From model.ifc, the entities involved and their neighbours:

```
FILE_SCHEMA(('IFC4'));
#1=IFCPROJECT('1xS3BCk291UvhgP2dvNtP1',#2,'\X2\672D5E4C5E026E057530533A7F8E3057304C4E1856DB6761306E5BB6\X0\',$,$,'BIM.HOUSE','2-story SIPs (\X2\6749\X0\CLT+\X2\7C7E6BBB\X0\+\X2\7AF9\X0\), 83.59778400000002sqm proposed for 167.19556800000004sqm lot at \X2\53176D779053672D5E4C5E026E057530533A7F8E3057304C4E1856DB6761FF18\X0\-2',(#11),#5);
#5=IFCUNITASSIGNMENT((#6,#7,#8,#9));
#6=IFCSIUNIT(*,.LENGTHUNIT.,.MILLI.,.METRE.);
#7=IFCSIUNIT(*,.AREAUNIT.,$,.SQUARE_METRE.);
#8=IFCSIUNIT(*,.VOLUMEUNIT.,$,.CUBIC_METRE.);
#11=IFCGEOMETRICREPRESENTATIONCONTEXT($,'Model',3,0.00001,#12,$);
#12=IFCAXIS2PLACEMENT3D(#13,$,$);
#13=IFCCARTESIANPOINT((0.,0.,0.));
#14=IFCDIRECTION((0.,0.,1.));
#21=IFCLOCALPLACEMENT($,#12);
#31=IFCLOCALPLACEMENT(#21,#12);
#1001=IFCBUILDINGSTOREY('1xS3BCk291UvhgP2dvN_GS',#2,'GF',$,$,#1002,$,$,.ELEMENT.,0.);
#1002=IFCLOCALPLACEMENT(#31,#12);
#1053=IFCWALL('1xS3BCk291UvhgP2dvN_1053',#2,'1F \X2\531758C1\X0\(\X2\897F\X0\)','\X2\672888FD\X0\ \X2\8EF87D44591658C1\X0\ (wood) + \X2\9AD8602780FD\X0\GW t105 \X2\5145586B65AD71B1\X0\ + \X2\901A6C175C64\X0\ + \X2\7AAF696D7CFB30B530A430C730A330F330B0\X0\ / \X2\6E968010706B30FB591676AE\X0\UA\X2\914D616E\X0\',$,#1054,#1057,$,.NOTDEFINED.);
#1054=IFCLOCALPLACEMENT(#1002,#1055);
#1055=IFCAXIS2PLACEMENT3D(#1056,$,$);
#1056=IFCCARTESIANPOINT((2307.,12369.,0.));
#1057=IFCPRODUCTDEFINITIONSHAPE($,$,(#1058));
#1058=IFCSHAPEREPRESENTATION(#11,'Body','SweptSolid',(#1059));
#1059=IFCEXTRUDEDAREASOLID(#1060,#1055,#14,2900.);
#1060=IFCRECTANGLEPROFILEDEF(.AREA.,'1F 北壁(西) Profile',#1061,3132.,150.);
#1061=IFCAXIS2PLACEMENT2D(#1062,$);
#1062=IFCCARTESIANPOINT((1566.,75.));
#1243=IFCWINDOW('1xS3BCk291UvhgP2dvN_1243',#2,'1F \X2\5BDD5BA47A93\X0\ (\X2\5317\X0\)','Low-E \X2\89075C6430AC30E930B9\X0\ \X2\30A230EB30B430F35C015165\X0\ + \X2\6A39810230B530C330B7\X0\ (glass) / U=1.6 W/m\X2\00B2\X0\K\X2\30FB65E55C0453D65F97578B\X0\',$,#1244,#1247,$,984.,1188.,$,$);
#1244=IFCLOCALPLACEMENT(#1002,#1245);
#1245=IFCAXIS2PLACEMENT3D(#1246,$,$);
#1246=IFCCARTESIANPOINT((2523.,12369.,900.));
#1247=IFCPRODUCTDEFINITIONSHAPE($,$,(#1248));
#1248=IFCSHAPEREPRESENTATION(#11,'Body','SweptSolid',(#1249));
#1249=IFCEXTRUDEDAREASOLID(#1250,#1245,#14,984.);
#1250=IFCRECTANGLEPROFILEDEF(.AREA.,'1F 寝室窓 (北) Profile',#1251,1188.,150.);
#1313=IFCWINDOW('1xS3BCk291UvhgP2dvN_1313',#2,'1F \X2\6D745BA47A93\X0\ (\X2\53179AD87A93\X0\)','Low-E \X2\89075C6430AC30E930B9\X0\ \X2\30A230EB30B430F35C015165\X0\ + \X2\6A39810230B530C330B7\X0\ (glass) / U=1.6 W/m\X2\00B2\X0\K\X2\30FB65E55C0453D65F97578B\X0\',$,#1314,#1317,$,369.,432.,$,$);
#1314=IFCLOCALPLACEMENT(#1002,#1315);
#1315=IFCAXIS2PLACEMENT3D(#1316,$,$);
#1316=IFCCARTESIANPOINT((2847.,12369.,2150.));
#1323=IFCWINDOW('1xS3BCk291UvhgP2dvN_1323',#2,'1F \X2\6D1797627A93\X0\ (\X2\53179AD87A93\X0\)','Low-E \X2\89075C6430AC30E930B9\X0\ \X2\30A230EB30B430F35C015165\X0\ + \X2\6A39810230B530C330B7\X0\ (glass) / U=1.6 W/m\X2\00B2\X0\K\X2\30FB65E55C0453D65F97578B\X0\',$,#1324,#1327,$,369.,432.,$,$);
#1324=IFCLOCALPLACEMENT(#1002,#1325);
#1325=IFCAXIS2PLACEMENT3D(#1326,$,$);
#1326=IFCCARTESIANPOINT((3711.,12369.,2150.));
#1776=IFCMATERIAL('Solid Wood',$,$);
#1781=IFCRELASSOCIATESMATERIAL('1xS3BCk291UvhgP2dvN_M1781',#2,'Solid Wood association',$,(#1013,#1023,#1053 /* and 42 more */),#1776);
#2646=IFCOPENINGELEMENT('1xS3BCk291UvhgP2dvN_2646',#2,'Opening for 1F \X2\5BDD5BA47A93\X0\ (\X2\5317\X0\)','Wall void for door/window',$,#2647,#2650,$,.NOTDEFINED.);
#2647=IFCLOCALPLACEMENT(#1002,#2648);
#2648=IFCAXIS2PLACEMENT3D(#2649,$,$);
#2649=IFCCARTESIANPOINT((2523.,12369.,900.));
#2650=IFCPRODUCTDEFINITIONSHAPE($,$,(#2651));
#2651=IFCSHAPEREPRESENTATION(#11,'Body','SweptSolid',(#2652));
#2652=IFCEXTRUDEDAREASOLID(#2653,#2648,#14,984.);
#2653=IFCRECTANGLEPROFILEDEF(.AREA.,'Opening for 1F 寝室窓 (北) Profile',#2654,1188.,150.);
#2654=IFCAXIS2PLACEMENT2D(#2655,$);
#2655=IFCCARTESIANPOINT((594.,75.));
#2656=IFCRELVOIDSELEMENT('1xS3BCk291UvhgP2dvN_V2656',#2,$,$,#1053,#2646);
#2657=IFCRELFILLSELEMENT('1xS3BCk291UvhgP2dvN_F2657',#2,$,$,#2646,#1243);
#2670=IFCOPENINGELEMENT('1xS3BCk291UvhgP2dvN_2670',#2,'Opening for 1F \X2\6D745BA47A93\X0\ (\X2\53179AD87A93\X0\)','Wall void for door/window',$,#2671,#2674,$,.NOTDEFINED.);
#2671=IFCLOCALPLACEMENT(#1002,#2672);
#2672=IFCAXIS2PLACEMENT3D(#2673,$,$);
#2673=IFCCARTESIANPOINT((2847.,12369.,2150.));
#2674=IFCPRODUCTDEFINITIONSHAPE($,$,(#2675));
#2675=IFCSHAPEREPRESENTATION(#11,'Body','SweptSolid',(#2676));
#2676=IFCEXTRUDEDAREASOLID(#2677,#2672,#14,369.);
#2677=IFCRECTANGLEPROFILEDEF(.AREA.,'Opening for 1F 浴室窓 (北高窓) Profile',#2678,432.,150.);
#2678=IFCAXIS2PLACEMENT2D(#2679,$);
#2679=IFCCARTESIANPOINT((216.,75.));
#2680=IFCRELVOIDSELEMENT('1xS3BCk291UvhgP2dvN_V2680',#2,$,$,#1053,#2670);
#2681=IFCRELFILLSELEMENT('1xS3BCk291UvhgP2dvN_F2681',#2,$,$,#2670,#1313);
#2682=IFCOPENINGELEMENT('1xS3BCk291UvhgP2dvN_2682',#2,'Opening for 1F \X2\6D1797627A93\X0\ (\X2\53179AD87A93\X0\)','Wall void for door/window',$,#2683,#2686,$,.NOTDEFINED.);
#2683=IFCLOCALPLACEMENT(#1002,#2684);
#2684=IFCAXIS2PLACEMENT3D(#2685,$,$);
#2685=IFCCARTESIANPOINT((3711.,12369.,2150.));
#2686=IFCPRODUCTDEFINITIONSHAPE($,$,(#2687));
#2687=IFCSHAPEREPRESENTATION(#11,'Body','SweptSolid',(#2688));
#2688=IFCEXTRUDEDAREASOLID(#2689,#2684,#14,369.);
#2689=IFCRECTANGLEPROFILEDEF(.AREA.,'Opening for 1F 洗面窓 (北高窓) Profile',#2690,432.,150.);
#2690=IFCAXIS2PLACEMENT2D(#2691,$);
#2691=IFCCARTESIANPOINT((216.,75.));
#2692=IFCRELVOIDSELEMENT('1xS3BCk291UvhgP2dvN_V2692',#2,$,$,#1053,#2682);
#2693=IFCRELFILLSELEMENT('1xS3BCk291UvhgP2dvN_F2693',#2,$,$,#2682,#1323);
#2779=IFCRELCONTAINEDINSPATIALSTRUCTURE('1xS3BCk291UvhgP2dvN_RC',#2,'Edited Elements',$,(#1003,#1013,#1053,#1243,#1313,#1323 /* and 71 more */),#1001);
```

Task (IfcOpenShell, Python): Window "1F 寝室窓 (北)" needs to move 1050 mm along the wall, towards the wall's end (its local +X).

```python
import ifcopenshell
import ifcopenshell.api.geometry
import ifcopenshell.util.placement
import ifcopenshell.util.unit

model = ifcopenshell.open("model.ifc")
unit_scale = ifcopenshell.util.unit.calculate_unit_scale(model)

window = model.by_guid("1xS3BCk291UvhgP2dvN_1243")
opening = window.FillsVoids[0].RelatingOpeningElement
wall = opening.VoidsElements[0].RelatingBuildingElement

wall_matrix = ifcopenshell.util.placement.get_local_placement(wall.ObjectPlacement)
shift = wall_matrix[:3, 0] * 1.05 / unit_scale
before = ifcopenshell.util.placement.get_local_placement(window.ObjectPlacement)[:3, 3].copy()

# The window is not placed relative to its opening, so move both.
for product in (opening, window):
    matrix = ifcopenshell.util.placement.get_local_placement(product.ObjectPlacement)
    matrix[:3, 3] += shift
    ifcopenshell.api.geometry.edit_object_placement(model, product=product, matrix=matrix, is_si=False)

after = ifcopenshell.util.placement.get_local_placement(window.ObjectPlacement)[:3, 3]
print("window moved by", (after - before).round(3) + 0.0)

model.write("model_updated.ifc")
```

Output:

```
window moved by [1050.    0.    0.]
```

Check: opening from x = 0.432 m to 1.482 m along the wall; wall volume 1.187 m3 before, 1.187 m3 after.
